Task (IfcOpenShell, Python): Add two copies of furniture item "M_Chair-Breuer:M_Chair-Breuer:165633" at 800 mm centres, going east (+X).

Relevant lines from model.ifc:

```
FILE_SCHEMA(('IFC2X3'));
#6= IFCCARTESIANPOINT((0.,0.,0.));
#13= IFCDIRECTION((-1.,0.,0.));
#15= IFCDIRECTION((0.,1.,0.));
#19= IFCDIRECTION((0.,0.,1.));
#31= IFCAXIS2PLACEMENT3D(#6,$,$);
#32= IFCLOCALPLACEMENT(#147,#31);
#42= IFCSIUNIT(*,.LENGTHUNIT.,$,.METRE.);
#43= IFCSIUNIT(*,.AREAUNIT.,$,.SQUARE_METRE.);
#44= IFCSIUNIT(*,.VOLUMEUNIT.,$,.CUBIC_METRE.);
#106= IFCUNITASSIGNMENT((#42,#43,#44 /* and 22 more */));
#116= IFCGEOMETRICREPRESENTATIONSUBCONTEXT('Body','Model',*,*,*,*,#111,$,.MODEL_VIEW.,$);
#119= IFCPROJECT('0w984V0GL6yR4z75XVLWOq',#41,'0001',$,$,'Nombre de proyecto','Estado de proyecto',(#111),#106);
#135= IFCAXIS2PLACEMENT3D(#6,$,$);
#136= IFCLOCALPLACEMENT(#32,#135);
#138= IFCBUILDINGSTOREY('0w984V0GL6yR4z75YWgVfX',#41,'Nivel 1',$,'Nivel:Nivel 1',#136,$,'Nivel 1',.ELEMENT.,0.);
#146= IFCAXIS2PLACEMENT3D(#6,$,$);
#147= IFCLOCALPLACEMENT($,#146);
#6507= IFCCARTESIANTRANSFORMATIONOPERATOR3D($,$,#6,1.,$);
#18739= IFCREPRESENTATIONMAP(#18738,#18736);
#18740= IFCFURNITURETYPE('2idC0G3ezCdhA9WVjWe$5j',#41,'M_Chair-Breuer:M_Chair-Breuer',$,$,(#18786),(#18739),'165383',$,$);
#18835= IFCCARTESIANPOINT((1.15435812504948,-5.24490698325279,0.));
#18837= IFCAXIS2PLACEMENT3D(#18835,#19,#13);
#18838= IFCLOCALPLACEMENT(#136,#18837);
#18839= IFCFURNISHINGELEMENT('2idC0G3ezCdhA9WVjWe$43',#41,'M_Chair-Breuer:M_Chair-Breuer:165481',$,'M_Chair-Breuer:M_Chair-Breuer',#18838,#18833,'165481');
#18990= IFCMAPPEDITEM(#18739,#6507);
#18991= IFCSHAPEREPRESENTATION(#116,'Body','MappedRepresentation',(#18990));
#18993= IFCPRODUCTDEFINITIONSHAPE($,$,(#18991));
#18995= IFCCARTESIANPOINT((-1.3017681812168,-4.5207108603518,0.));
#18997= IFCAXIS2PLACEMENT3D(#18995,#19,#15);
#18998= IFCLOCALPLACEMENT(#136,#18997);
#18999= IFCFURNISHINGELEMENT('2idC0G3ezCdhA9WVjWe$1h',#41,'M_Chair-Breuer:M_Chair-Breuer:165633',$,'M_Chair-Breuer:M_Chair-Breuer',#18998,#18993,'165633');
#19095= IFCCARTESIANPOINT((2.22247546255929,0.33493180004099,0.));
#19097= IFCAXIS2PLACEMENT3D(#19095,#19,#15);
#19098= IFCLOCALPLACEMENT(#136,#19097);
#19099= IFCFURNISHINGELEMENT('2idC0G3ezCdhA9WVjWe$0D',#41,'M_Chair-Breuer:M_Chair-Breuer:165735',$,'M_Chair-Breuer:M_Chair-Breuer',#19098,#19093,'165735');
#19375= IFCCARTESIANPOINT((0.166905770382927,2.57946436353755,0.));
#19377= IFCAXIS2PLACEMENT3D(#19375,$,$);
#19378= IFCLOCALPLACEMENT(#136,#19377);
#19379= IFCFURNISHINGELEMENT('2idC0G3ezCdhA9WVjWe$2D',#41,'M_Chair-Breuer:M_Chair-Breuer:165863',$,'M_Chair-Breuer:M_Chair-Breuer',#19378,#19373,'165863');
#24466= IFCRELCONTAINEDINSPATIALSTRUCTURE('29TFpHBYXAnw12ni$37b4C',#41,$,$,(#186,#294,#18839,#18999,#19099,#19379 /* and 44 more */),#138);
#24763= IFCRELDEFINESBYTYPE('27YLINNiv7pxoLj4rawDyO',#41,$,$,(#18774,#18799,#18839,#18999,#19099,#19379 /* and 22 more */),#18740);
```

```python
import numpy as np
import ifcopenshell
import ifcopenshell.api.geometry
import ifcopenshell.api.root
import ifcopenshell.util.element
import ifcopenshell.util.placement
import ifcopenshell.util.unit

model = ifcopenshell.open("model.ifc")
unit_scale = ifcopenshell.util.unit.calculate_unit_scale(model)


def reuse_history(source, copy):
    """copy_class also copies each property set's owner history, people and application; keep the originals."""
    for rel in copy.IsDefinedBy:
        if rel.is_a("IfcRelDefinesByProperties") and (history := rel.RelatingPropertyDefinition.OwnerHistory):
            rel.RelatingPropertyDefinition.OwnerHistory = source.OwnerHistory
            ifcopenshell.util.element.remove_deep2(model, history)


source = model.by_guid("2idC0G3ezCdhA9WVjWe$1h")
base = ifcopenshell.util.placement.get_local_placement(source.ObjectPlacement)
step = np.array([1.0, 0.0, 0.0]) * 0.8 / unit_scale

for i in range(1, 3):
    copy = ifcopenshell.api.root.copy_class(model, product=source)
    copy.Representation = ifcopenshell.util.element.copy_deep(
        model, source.Representation, exclude=["IfcGeometricRepresentationContext", "IfcRepresentationMap"]
    )
    copy.Name = "M_Chair-Breuer:M_Chair-Breuer"
    copy.Tag = None
    reuse_history(source, copy)
    matrix = base.copy()
    matrix[:3, 3] += i * step
    print("added at", matrix[:3, 3].round(3) + 0.0)
    ifcopenshell.api.geometry.edit_object_placement(model, product=copy, matrix=matrix, is_si=False)

model.write("model_v2.ifc")
```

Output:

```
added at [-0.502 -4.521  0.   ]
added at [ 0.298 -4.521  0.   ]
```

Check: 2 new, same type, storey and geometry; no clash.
